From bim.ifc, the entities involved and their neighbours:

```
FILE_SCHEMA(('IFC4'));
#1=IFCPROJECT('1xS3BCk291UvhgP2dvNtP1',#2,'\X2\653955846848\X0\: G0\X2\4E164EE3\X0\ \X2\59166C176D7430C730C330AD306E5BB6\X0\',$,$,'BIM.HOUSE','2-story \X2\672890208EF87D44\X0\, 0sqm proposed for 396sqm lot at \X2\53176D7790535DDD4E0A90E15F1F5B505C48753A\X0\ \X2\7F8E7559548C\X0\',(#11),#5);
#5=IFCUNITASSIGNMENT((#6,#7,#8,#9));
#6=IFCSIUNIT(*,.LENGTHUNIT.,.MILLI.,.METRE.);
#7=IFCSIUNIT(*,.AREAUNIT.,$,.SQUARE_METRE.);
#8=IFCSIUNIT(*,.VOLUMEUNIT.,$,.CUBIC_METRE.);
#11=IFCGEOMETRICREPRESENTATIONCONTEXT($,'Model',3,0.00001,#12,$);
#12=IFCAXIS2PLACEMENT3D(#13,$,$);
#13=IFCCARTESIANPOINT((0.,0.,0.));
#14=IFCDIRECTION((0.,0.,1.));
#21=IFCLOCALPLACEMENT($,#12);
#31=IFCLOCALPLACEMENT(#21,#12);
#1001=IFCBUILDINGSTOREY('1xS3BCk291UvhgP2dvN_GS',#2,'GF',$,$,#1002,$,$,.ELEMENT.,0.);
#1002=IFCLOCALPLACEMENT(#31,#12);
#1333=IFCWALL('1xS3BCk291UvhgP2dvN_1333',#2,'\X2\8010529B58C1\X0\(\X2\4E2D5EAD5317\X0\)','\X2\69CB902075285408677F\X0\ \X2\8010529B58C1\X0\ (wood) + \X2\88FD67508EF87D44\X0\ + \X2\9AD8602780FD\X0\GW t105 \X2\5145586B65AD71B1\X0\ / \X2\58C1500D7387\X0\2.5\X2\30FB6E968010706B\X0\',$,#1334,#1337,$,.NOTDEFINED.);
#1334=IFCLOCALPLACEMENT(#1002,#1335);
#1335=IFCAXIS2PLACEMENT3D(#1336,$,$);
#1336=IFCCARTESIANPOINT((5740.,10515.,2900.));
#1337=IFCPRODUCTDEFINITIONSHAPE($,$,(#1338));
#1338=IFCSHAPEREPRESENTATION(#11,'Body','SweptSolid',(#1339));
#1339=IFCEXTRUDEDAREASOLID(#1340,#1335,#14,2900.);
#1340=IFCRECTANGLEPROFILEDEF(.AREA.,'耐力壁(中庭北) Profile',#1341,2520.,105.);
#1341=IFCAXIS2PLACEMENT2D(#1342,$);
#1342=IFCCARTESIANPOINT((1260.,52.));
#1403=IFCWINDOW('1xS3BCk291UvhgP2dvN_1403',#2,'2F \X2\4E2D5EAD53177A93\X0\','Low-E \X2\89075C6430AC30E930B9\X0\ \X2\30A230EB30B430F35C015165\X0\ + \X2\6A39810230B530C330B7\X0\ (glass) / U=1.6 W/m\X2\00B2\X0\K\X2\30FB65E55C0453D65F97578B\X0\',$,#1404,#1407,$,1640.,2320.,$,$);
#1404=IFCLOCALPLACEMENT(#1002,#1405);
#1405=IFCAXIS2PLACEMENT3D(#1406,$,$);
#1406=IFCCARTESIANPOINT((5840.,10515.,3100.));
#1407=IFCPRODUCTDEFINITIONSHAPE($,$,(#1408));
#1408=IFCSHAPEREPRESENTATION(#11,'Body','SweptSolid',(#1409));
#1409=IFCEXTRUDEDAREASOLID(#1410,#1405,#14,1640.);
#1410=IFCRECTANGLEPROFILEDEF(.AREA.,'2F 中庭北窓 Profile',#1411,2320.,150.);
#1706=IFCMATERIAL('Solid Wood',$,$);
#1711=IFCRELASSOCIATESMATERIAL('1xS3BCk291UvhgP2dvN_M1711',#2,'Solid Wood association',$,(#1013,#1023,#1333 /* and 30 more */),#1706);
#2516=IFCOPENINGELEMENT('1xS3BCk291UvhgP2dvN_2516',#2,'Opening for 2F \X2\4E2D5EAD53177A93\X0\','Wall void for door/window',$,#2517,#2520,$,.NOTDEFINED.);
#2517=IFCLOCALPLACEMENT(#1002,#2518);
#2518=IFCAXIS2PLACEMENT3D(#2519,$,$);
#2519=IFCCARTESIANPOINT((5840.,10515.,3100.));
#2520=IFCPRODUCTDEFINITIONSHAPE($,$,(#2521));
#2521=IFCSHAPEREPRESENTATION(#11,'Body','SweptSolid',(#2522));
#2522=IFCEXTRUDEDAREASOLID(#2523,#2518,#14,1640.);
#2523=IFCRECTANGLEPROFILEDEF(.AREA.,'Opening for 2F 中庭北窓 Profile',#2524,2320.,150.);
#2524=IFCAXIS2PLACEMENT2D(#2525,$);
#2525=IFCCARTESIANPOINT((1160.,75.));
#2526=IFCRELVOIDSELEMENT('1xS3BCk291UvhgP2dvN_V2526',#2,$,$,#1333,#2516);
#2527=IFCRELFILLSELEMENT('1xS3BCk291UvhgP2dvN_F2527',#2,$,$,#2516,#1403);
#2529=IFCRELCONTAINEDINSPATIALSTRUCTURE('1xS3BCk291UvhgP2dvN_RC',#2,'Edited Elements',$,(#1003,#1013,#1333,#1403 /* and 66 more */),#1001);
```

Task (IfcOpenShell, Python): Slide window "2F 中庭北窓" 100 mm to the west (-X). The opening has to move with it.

```python
import ifcopenshell
import ifcopenshell.api.geometry
import ifcopenshell.util.placement

model = ifcopenshell.open("bim.ifc")

window = model.by_id(1403)
opening = window.FillsVoids[0].RelatingOpeningElement
wall = opening.VoidsElements[0].RelatingBuildingElement

wall_matrix = ifcopenshell.util.placement.get_local_placement(wall.ObjectPlacement)
shift = wall_matrix[:3, 0] * -100.0
before = ifcopenshell.util.placement.get_local_placement(window.ObjectPlacement)[:3, 3].copy()

# The window is not placed relative to its opening, so move both.
for product in (opening, window):
    matrix = ifcopenshell.util.placement.get_local_placement(product.ObjectPlacement)
    matrix[:3, 3] += shift
    ifcopenshell.api.geometry.edit_object_placement(model, product=product, matrix=matrix, is_si=False)

after = ifcopenshell.util.placement.get_local_placement(window.ObjectPlacement)[:3, 3]
print("window moved by", (after - before).round(3) + 0.0)

model.write("bim_updated.ifc")
```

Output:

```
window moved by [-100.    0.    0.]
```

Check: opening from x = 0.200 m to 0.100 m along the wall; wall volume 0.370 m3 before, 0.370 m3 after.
